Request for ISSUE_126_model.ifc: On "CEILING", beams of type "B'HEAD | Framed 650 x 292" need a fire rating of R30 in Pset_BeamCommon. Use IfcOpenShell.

First a look at what the model holds.

```python
import ifcopenshell
import ifcopenshell.util.element

model = ifcopenshell.open("ISSUE_126_model.ifc")
print(model.schema)
storey = next(s for s in model.by_type("IfcBuildingStorey") if s.Name == "CEILING")
beams = [e for e in ifcopenshell.util.element.get_decomposition(storey) if e.is_a("IfcBeam")]
seen = {}
for e in beams:
    element_type = ifcopenshell.util.element.get_type(e)
    key = (element_type.Name if element_type != e and element_type else None, ifcopenshell.util.element.get_pset(e, "Pset_BeamCommon", "FireRating"))
    seen[key] = seen.get(key, 0) + 1
for (name, value), count in sorted(seen.items(), key=str):
    print(count, "x", name, "|", value)
```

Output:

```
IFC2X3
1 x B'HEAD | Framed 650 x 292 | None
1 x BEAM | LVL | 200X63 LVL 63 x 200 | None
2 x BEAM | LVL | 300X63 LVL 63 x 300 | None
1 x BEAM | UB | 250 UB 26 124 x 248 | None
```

```python
import ifcopenshell
import ifcopenshell.api.pset
import ifcopenshell.util.element

model = ifcopenshell.open("ISSUE_126_model.ifc")

storey = next(s for s in model.by_type("IfcBuildingStorey") if s.Name == "CEILING")
beams = [e for e in ifcopenshell.util.element.get_decomposition(storey) if e.is_a("IfcBeam")]

count = 0
for e in beams:
    element_type = ifcopenshell.util.element.get_type(e)
    if element_type in (None, e) or element_type.Name != "B'HEAD | Framed 650 x 292":
        continue
    # add_pset returns the element's existing set when there is one.
    pset = ifcopenshell.api.pset.add_pset(model, product=e, name="Pset_BeamCommon")
    ifcopenshell.api.pset.edit_pset(model, pset=pset, properties={"FireRating": "R30"})
    count += 1

print(count, "beams updated")

model.write("ISSUE_126_model_edited.ifc")
```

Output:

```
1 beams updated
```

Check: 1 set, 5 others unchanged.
